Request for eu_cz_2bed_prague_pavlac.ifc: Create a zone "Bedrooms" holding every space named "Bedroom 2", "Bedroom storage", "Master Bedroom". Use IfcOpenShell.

First a look at what the model holds.

```python
import ifcopenshell

model = ifcopenshell.open("eu_cz_2bed_prague_pavlac.ifc")
print(model.schema)
seen = {}
for space in model.by_type("IfcSpace"):
    seen[space.LongName] = seen.get(space.LongName, 0) + 1
for name, count in sorted(seen.items(), key=str):
    print(count, "x", name)
print("zones:", [z.Name for z in model.by_type("IfcZone")][:20])
```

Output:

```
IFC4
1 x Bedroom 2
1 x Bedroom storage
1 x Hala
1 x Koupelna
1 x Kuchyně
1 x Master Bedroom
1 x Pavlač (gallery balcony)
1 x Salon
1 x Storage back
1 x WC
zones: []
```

```python
import ifcopenshell
import ifcopenshell.api.group
import ifcopenshell.api.root

model = ifcopenshell.open("eu_cz_2bed_prague_pavlac.ifc")

names = {"Bedroom 2", "Bedroom storage", "Master Bedroom"}
spaces = [s for s in model.by_type("IfcSpace") if s.LongName in names]

zone = ifcopenshell.api.root.create_entity(model, ifc_class="IfcZone", name="Bedrooms")
ifcopenshell.api.group.assign_group(model, products=spaces, group=zone)
print(len(spaces), "spaces in", zone.Name)

model.write("eu_cz_2bed_prague_pavlac-out.ifc")
```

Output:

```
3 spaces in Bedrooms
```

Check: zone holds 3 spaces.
